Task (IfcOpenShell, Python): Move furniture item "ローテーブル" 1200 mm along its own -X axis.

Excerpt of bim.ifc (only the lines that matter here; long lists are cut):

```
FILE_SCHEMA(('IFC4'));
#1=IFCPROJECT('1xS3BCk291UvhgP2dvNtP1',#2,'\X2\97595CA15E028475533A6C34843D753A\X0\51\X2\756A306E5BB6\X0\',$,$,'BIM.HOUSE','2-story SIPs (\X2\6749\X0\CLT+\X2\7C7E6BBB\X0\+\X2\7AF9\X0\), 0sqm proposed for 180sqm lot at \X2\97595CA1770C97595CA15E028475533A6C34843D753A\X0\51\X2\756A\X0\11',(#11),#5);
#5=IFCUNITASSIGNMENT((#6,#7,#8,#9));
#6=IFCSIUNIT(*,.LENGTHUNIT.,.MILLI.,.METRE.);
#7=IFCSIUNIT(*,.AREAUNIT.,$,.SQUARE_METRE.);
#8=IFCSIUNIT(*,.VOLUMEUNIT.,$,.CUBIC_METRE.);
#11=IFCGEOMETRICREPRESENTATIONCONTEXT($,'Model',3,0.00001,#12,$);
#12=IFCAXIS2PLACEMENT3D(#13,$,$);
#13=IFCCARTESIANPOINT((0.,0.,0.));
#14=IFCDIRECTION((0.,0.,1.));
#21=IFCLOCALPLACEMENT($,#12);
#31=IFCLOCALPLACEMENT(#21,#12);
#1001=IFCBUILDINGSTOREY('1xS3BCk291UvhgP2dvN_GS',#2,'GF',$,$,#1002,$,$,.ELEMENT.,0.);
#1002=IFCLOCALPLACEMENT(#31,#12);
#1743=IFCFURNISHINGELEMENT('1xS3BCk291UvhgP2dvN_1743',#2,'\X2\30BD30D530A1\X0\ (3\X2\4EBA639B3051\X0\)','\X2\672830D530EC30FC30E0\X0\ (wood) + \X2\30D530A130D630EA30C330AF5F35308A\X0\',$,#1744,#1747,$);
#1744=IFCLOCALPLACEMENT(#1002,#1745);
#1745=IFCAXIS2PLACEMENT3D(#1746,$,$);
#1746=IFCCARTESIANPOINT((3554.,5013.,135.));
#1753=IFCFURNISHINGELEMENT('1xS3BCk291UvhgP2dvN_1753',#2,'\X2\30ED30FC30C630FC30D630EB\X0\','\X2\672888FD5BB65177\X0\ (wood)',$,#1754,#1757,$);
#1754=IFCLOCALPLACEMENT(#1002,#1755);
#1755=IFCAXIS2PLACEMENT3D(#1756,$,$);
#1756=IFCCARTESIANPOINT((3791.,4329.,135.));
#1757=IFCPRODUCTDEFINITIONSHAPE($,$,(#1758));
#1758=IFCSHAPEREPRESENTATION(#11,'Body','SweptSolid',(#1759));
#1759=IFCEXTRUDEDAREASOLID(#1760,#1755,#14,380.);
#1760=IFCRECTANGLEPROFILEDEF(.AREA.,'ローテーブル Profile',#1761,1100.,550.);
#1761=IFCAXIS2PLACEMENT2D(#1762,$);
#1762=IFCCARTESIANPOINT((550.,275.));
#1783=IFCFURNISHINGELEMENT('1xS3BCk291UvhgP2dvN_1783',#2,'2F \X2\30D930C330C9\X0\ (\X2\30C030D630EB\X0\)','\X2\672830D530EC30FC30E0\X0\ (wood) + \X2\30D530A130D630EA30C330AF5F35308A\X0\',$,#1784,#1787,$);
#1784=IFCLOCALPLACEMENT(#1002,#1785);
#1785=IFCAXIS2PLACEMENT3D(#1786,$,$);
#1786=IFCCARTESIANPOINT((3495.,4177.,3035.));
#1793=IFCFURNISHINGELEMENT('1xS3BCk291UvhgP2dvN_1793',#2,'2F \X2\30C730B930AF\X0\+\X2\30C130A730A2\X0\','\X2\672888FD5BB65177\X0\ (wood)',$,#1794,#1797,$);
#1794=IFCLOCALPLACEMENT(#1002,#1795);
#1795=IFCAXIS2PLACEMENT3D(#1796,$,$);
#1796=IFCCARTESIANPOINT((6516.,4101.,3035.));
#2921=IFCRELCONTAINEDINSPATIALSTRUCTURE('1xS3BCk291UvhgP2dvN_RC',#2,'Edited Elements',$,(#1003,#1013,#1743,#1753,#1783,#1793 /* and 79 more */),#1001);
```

```python
import ifcopenshell
import ifcopenshell.api.geometry
import ifcopenshell.util.placement
import ifcopenshell.util.unit

model = ifcopenshell.open("bim.ifc")
unit_scale = ifcopenshell.util.unit.calculate_unit_scale(model)

item = model.by_guid("1xS3BCk291UvhgP2dvN_1753")
matrix = ifcopenshell.util.placement.get_local_placement(item.ObjectPlacement)
matrix[:3, 3] -= matrix[:3, 0] * 1.2 / unit_scale
ifcopenshell.api.geometry.edit_object_placement(model, product=item, matrix=matrix, is_si=False)

print(ifcopenshell.util.placement.get_local_placement(item.ObjectPlacement).round(3) + 0.0)

model.write("bim_rev.ifc")
```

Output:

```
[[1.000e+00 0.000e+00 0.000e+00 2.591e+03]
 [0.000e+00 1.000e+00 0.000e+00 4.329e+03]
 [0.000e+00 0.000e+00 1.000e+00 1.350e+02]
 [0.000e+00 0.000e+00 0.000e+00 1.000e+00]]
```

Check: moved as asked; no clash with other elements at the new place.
